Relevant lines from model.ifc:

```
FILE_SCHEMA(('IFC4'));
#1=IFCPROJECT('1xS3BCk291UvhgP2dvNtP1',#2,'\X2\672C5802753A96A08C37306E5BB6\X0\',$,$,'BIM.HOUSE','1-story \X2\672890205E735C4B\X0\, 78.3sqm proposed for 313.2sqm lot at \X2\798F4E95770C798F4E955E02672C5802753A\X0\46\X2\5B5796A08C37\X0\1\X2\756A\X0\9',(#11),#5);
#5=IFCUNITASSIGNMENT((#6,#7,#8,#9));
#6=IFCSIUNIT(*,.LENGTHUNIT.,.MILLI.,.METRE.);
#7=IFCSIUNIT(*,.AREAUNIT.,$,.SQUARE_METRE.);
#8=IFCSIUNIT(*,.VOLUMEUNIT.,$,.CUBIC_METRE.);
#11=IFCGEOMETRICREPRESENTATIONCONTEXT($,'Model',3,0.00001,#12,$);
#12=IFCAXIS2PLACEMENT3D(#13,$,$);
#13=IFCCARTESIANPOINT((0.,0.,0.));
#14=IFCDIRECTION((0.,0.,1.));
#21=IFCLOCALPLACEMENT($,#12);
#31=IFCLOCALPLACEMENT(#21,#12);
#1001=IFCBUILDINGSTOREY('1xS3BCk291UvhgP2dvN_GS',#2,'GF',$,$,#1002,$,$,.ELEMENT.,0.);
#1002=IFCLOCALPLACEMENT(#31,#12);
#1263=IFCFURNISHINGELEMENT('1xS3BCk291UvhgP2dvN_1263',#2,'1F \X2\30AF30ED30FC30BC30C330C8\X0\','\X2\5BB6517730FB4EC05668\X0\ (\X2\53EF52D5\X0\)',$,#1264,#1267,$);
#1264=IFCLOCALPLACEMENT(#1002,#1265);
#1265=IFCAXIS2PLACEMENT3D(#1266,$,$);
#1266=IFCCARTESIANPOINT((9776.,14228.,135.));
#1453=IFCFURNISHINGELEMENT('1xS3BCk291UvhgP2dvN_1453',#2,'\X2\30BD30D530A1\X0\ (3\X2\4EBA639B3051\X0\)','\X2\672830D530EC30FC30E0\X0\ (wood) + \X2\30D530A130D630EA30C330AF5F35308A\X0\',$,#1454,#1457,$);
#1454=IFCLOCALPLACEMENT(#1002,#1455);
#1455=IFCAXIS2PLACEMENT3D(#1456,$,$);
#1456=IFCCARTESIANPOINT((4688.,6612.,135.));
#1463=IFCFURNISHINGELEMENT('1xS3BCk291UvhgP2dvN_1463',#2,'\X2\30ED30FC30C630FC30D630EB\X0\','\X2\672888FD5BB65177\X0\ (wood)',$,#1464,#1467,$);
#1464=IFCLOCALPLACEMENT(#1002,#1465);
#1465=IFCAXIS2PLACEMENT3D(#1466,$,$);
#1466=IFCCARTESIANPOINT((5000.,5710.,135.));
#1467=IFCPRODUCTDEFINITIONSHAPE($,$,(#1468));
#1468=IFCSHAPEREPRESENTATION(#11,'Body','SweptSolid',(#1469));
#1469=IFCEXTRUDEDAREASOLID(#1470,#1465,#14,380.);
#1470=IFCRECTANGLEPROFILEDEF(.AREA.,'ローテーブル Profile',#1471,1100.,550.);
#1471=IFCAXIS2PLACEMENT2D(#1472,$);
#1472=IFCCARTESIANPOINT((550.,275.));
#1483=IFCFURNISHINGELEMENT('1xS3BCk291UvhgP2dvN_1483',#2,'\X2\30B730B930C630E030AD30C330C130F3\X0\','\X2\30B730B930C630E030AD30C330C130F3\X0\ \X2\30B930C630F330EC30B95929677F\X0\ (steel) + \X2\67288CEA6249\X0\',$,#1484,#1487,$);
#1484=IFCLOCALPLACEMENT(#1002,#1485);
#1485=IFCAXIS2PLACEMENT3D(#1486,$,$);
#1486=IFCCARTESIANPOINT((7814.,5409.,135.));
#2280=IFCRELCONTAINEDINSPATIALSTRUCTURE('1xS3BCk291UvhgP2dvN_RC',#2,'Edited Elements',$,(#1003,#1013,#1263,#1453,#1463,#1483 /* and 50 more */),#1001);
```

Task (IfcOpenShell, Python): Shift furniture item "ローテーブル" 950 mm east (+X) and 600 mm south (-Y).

```python
import ifcopenshell
import ifcopenshell.api.geometry
import ifcopenshell.util.placement
import ifcopenshell.util.unit

model = ifcopenshell.open("model.ifc")
unit_scale = ifcopenshell.util.unit.calculate_unit_scale(model)

item = model.by_guid("1xS3BCk291UvhgP2dvN_1463")
matrix = ifcopenshell.util.placement.get_local_placement(item.ObjectPlacement)
matrix[0, 3] += 0.95 / unit_scale
matrix[1, 3] -= 0.6 / unit_scale
ifcopenshell.api.geometry.edit_object_placement(model, product=item, matrix=matrix, is_si=False)

print(ifcopenshell.util.placement.get_local_placement(item.ObjectPlacement).round(3) + 0.0)

model.write("model_updated.ifc")
```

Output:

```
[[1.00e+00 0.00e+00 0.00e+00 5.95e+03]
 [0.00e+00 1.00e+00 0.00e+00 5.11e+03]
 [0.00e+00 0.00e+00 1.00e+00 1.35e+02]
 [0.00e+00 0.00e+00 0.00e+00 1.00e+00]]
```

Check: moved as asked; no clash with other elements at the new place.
